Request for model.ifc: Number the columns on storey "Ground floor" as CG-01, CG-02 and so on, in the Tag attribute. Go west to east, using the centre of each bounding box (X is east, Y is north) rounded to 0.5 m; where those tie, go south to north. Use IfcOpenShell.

First a look at what the model holds.

```python
import ifcopenshell
import ifcopenshell.util.element
import ifcopenshell.util.placement

model = ifcopenshell.open("model.ifc")
print(model.schema)
storey = next(s for s in model.by_type("IfcBuildingStorey") if s.Name == "Ground floor")
columns = [e for e in ifcopenshell.util.element.get_decomposition(storey) if e.is_a("IfcColumn")]
for e in sorted(columns, key=lambda e: e.id()):
    origin = ifcopenshell.util.placement.get_local_placement(e.ObjectPlacement)[:3, 3]
    print(e.id(), e.Tag, e.Name, origin.round(2) + 0.0, sep=" | ")
```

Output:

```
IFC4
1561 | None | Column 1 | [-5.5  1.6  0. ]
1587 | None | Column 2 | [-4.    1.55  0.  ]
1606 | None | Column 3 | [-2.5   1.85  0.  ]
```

```python
import ifcopenshell
import ifcopenshell.geom
import ifcopenshell.util.element
import ifcopenshell.util.shape

model = ifcopenshell.open("model.ifc")
settings = ifcopenshell.geom.settings()
settings.set("use-world-coords", True)


def centre(element):
    shape = ifcopenshell.geom.create_shape(settings, element)
    return ifcopenshell.util.shape.get_bbox_centroid(shape.geometry)


storey = next(s for s in model.by_type("IfcBuildingStorey") if s.Name == "Ground floor")
columns = [e for e in ifcopenshell.util.element.get_decomposition(storey) if e.is_a("IfcColumn")]

# Insertion points can sit at a corner or the storey origin, so sort by the geometry (in metres).
centres = {e: centre(e) for e in columns}
columns.sort(key=lambda e: (round(centres[e][0] / 0.5), centres[e][1]))

for i, e in enumerate(columns, start=1):
    number = f"CG-{i:02d}"
    e.Tag = number
    print(e.id(), number)

model.write("model_updated.ifc")
```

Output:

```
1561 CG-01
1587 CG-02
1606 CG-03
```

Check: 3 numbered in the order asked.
